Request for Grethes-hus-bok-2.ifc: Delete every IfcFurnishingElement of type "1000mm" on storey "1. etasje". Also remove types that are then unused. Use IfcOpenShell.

First a look at what the model holds.

```python
import ifcopenshell
import ifcopenshell.util.element

model = ifcopenshell.open("Grethes-hus-bok-2.ifc")
print(model.schema)
storey = next(s for s in model.by_type("IfcBuildingStorey") if s.Name == "1. etasje")
furniture = [e for e in ifcopenshell.util.element.get_decomposition(storey) if e.is_a("IfcFurnishingElement")]
seen = {}
for e in furniture:
    element_type = ifcopenshell.util.element.get_type(e)
    name = element_type.Name if element_type not in (None, e) else None
    seen[name] = seen.get(name, 0) + 1
for name, count in sorted(seen.items(), key=str):
    print(count, "x", name)
```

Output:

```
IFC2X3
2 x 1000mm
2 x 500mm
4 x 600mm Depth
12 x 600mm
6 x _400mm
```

```python
import ifcopenshell
import ifcopenshell.api.root
import ifcopenshell.util.element

model = ifcopenshell.open("Grethes-hus-bok-2.ifc")

storey = next(s for s in model.by_type("IfcBuildingStorey") if s.Name == "1. etasje")
furniture = [e for e in ifcopenshell.util.element.get_decomposition(storey) if e.is_a("IfcFurnishingElement")]
targets = [e for e in furniture if (t := ifcopenshell.util.element.get_type(e)) not in (None, e) and t.Name == "1000mm"]
types = {ifcopenshell.util.element.get_type(e) for e in targets} - {None, *targets}

for e in targets:
    ifcopenshell.api.root.remove_product(model, product=e)
print(len(targets), "removed")

unused = [t for t in types if not ifcopenshell.util.element.get_types(t)]
for t in unused:
    ifcopenshell.api.root.remove_product(model, product=t)
print(len(unused), "unused types removed")

model.write("Grethes-hus-bok-2-out.ifc")
```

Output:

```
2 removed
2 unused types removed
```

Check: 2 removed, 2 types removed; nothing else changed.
